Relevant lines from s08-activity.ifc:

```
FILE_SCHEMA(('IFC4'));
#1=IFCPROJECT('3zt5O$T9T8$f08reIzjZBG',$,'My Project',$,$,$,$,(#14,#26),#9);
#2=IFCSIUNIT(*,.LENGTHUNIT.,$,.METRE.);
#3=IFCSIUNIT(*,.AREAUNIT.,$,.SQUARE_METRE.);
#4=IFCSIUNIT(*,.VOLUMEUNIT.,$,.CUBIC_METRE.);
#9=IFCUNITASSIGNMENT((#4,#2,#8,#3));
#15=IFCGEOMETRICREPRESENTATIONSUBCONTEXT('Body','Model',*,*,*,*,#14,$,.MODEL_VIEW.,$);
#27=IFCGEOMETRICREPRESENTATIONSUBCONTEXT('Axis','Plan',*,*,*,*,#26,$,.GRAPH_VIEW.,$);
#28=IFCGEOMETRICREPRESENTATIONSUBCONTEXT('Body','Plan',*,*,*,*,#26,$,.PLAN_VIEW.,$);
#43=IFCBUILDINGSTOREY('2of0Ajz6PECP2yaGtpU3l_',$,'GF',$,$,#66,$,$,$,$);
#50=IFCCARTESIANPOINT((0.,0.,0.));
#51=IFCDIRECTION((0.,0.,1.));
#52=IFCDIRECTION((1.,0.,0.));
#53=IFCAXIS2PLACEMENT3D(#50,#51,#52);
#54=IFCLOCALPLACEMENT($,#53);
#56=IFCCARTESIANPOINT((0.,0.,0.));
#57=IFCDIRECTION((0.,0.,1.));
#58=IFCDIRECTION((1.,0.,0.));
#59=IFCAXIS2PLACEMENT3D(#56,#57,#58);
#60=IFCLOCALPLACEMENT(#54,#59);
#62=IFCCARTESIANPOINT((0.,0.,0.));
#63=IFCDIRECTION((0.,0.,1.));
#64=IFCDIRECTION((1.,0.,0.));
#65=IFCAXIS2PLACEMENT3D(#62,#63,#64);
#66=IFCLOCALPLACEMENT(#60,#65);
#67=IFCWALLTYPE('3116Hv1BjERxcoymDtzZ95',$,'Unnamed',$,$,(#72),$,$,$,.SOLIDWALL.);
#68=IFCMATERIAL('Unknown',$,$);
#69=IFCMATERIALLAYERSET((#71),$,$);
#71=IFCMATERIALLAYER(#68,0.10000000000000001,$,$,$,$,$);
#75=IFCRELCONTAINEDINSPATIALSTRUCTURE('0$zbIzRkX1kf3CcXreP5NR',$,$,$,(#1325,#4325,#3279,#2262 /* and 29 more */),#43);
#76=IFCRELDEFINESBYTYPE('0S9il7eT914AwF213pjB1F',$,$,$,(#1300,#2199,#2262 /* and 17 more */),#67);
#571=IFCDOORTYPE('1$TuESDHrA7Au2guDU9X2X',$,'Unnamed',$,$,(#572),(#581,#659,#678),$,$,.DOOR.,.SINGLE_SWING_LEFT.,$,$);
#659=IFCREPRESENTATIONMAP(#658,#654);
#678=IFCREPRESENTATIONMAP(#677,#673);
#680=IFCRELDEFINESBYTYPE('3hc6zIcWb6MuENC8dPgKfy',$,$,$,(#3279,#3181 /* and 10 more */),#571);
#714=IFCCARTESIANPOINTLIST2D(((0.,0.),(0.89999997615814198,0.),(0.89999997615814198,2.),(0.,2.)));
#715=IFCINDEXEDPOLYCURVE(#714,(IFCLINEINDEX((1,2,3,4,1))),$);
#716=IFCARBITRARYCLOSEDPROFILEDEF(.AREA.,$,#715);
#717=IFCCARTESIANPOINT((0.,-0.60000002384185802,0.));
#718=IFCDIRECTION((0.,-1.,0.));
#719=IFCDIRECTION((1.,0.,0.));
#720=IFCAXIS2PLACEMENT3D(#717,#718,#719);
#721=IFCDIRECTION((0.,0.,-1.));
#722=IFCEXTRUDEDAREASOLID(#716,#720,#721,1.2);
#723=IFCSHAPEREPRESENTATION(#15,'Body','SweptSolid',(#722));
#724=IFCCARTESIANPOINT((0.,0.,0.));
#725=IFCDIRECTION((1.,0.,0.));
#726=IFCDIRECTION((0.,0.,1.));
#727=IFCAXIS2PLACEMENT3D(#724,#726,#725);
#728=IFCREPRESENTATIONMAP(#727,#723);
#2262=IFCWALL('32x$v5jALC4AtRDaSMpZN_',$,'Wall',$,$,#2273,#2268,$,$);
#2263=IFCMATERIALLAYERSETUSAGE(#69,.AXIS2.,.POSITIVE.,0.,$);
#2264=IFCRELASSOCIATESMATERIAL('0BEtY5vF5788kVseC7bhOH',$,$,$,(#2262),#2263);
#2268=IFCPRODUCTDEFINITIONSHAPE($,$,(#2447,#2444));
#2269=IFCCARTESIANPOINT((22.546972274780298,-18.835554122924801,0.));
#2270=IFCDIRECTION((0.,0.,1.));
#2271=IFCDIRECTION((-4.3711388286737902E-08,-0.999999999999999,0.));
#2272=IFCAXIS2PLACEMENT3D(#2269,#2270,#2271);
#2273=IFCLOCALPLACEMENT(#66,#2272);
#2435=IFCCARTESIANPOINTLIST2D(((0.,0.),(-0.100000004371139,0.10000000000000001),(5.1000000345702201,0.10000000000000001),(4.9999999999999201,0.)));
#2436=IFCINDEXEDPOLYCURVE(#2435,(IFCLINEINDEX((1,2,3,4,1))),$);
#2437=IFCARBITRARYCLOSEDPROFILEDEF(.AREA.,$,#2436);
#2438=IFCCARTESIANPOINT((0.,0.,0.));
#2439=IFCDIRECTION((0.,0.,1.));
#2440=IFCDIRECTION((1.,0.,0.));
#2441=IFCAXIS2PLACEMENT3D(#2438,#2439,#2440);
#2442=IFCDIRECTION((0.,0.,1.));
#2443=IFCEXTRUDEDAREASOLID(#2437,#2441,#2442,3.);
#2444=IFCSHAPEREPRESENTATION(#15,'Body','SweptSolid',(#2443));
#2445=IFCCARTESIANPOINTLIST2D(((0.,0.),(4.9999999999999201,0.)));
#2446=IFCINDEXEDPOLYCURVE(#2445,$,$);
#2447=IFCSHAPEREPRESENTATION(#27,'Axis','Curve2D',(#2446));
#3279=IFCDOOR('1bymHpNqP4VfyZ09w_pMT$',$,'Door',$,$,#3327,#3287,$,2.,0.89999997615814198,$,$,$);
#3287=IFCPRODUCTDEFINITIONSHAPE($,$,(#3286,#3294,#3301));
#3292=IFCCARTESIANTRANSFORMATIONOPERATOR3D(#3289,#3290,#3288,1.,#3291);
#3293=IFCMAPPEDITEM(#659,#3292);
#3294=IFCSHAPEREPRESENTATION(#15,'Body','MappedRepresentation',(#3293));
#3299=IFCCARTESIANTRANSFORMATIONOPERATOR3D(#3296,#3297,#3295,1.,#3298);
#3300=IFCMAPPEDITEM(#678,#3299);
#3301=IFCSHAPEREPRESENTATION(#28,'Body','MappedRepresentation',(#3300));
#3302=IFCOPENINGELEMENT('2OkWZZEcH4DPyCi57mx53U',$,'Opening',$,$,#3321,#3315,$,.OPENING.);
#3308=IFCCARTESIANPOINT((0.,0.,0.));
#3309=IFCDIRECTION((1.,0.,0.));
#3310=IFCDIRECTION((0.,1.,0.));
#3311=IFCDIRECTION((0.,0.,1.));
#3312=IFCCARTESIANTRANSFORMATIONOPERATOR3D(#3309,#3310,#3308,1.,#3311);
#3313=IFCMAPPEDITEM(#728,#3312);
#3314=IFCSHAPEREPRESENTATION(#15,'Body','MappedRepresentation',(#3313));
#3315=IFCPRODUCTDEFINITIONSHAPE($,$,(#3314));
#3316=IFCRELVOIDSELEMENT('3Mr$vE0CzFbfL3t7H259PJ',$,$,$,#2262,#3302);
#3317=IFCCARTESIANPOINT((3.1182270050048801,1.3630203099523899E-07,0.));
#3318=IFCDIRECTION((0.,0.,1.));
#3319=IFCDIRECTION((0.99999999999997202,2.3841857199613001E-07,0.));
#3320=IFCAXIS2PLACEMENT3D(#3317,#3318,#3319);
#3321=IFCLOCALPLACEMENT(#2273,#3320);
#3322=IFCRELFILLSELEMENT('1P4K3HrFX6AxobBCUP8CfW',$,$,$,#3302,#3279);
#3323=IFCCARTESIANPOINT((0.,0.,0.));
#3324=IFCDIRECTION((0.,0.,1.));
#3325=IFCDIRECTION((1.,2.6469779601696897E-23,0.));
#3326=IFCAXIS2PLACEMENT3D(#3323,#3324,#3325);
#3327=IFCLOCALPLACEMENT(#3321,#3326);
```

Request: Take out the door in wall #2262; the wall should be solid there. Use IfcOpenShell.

```python
import ifcopenshell
import ifcopenshell.api.feature
import ifcopenshell.api.root
import ifcopenshell.geom
import ifcopenshell.util.shape

model = ifcopenshell.open("s08-activity.ifc")
settings = ifcopenshell.geom.settings()


def volume(element):
    """Net volume in cubic metres, openings subtracted."""
    shape = ifcopenshell.geom.create_shape(settings, element)
    return ifcopenshell.util.shape.get_volume(shape.geometry)


door = model.by_guid("1bymHpNqP4VfyZ09w_pMT$")
opening = door.FillsVoids[0].RelatingOpeningElement
wall = opening.VoidsElements[0].RelatingBuildingElement
before = volume(wall)

ifcopenshell.api.root.remove_product(model, product=door)
ifcopenshell.api.feature.remove_feature(model, feature=opening)

after = volume(wall)

print(f"wall volume {before:.3f} -> {after:.3f} m3")

model.write("s08-activity-out.ifc")
```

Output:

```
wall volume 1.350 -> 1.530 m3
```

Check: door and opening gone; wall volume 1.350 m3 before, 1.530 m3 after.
